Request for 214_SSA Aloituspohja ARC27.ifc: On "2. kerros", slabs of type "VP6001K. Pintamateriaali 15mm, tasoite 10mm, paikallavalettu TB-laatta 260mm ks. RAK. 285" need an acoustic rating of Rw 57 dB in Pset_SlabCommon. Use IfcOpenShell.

First a look at what the model holds.

```python
import ifcopenshell
import ifcopenshell.util.element

model = ifcopenshell.open("214_SSA Aloituspohja ARC27.ifc")
print(model.schema)
storey = next(s for s in model.by_type("IfcBuildingStorey") if s.Name == "2. kerros")
slabs = [e for e in ifcopenshell.util.element.get_decomposition(storey) if e.is_a("IfcSlab")]
seen = {}
for e in slabs:
    element_type = ifcopenshell.util.element.get_type(e)
    key = (element_type.Name if element_type != e and element_type else None, ifcopenshell.util.element.get_pset(e, "Pset_SlabCommon", "AcousticRating"))
    seen[key] = seen.get(key, 0) + 1
for (name, value), count in sorted(seen.items(), key=str):
    print(count, "x", name, "|", value)
```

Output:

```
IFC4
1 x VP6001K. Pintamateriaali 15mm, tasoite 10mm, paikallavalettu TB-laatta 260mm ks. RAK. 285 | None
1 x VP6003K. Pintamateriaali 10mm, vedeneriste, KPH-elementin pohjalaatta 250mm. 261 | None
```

```python
import ifcopenshell
import ifcopenshell.api.pset
import ifcopenshell.util.element

model = ifcopenshell.open("214_SSA Aloituspohja ARC27.ifc")

storey = next(s for s in model.by_type("IfcBuildingStorey") if s.Name == "2. kerros")
slabs = [e for e in ifcopenshell.util.element.get_decomposition(storey) if e.is_a("IfcSlab")]

count = 0
for e in slabs:
    element_type = ifcopenshell.util.element.get_type(e)
    if element_type in (None, e) or element_type.Name != "VP6001K. Pintamateriaali 15mm, tasoite 10mm, paikallavalettu TB-laatta 260mm ks. RAK. 285":
        continue
    # add_pset returns the element's existing set when there is one.
    pset = ifcopenshell.api.pset.add_pset(model, product=e, name="Pset_SlabCommon")
    ifcopenshell.api.pset.edit_pset(model, pset=pset, properties={"AcousticRating": "Rw 57 dB"})
    count += 1

print(count, "slabs updated")

model.write("214_SSA Aloituspohja ARC27-out.ifc")
```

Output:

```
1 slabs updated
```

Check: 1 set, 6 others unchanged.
